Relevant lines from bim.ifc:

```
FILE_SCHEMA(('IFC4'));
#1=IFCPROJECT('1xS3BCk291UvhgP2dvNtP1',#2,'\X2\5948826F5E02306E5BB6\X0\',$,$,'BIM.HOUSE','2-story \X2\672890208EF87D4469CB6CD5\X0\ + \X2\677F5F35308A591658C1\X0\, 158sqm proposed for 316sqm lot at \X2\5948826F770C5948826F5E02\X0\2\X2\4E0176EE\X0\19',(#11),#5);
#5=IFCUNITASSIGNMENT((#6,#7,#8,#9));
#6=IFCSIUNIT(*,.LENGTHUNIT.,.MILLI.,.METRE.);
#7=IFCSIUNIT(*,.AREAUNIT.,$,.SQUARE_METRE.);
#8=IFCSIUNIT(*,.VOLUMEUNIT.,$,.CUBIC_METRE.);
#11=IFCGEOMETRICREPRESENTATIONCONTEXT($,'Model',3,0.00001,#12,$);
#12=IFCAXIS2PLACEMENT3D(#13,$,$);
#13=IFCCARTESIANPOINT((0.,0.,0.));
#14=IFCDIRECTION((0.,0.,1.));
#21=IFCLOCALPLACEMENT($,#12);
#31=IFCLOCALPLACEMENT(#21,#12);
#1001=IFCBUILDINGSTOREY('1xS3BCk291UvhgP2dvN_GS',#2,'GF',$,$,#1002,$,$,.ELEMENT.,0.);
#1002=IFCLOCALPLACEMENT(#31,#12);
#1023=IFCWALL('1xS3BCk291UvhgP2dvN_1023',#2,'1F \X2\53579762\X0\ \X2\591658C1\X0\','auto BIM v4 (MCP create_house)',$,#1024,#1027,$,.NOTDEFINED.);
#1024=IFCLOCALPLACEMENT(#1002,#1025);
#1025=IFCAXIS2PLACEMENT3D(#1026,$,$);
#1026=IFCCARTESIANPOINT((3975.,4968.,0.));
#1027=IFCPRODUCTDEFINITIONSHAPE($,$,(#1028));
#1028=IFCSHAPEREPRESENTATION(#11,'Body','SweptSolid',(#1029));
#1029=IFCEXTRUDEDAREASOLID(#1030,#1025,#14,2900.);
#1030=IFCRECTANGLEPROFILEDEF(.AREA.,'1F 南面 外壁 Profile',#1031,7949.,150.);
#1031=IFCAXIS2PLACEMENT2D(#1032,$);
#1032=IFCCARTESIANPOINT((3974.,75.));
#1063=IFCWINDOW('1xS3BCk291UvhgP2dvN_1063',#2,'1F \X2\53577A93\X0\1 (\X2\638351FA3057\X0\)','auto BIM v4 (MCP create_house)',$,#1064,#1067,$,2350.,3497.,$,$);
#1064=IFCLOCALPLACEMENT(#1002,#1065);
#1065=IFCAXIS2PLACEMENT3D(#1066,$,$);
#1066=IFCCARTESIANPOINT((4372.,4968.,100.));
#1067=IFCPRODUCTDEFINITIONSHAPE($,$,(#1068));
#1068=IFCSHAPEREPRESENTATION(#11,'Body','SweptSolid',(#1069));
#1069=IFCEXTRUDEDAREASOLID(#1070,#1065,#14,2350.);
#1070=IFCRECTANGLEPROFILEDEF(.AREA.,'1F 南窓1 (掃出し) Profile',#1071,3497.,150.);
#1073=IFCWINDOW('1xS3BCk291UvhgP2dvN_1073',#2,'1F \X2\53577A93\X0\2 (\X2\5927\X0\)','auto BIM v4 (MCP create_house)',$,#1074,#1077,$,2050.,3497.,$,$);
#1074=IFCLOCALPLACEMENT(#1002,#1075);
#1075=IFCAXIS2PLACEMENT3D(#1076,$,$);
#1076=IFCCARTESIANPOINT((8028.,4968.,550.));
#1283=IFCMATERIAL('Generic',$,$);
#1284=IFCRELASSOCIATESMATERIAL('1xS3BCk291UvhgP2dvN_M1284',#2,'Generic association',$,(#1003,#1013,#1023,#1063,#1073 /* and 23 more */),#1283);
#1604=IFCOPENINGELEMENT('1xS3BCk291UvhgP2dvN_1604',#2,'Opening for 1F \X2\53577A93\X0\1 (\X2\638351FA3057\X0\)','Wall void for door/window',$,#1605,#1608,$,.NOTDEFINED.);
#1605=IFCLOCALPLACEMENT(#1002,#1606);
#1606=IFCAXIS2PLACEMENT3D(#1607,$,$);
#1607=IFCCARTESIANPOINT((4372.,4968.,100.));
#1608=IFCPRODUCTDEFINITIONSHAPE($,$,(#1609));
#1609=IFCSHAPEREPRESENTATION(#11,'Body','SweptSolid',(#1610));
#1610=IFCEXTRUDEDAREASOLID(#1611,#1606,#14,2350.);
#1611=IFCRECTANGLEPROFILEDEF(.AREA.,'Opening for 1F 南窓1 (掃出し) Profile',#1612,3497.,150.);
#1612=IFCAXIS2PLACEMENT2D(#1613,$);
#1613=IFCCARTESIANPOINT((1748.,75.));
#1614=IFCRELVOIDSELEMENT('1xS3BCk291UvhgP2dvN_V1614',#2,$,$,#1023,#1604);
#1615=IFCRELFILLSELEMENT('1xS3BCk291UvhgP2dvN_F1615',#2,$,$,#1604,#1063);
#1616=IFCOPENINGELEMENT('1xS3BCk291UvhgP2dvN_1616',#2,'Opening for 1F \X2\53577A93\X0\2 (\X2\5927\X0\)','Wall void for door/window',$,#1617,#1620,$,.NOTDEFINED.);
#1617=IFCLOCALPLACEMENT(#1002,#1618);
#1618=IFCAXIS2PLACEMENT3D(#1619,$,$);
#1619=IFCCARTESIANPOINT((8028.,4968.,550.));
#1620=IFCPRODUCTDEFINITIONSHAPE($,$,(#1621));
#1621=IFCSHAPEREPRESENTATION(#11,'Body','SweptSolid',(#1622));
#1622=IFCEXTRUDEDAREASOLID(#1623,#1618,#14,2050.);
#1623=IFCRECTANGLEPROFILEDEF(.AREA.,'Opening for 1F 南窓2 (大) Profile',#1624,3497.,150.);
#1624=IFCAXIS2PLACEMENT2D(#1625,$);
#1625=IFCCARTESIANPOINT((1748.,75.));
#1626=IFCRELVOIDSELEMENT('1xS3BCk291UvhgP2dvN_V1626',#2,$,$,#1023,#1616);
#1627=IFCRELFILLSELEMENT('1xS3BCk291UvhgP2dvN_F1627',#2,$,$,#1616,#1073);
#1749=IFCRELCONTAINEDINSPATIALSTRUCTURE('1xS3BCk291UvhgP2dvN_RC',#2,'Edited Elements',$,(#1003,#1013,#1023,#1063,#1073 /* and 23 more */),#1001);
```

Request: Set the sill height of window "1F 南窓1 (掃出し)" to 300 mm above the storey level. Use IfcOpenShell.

```python
import numpy as np
import ifcopenshell
import ifcopenshell.api.geometry
import ifcopenshell.geom
import ifcopenshell.util.element
import ifcopenshell.util.placement
import ifcopenshell.util.shape
import ifcopenshell.util.unit

model = ifcopenshell.open("bim.ifc")
unit_scale = ifcopenshell.util.unit.calculate_unit_scale(model)

window = model.by_id(1063)
opening = window.FillsVoids[0].RelatingOpeningElement
storey = ifcopenshell.util.element.get_container(window, ifc_class="IfcBuildingStorey")
level = ifcopenshell.util.placement.get_local_placement(storey.ObjectPlacement)[2, 3]

# The opening's origin need not be at the sill, so measure its lowest point.
shape = ifcopenshell.geom.create_shape(ifcopenshell.geom.settings(), opening)
bottom = ifcopenshell.util.shape.get_shape_bottom_elevation(shape, shape.geometry) / unit_scale
dz = level + 0.3 / unit_scale - bottom

shift = np.array([0.0, 0.0, dz])
# The window is not placed relative to its opening, so move both.
for product in (opening, window):
    matrix = ifcopenshell.util.placement.get_local_placement(product.ObjectPlacement)
    matrix[:3, 3] += shift
    ifcopenshell.api.geometry.edit_object_placement(model, product=product, matrix=matrix, is_si=False)

print(f"moved by {dz * unit_scale:+.3f} m")

model.write("bim_v2.ifc")
```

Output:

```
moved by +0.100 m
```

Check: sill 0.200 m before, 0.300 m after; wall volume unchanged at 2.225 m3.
